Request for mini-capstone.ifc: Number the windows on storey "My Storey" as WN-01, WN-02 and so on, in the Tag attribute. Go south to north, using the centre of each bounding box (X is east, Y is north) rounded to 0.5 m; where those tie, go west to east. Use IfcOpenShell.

First a look at what the model holds.

```python
import ifcopenshell
import ifcopenshell.util.element
import ifcopenshell.util.placement

model = ifcopenshell.open("mini-capstone.ifc")
print(model.schema)
storey = next(s for s in model.by_type("IfcBuildingStorey") if s.Name == "My Storey")
windows = [e for e in ifcopenshell.util.element.get_decomposition(storey) if e.is_a("IfcWindow")]
for e in sorted(windows, key=lambda e: e.id()):
    origin = ifcopenshell.util.placement.get_local_placement(e.ObjectPlacement)[:3, 3]
    print(e.id(), e.Tag, e.Name, origin.round(2) + 0.0, sep=" | ")
```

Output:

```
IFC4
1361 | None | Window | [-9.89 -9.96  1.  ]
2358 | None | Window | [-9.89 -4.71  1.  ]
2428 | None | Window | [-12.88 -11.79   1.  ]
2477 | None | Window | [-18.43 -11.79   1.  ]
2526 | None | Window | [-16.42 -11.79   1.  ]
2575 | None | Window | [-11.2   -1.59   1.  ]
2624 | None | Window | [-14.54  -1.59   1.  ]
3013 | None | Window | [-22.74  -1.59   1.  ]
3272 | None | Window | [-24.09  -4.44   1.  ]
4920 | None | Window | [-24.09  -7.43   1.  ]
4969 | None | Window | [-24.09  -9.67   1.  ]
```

```python
import ifcopenshell
import ifcopenshell.geom
import ifcopenshell.util.element
import ifcopenshell.util.shape

model = ifcopenshell.open("mini-capstone.ifc")
settings = ifcopenshell.geom.settings()
settings.set("use-world-coords", True)


def centre(element):
    shape = ifcopenshell.geom.create_shape(settings, element)
    return ifcopenshell.util.shape.get_bbox_centroid(shape.geometry)


storey = next(s for s in model.by_type("IfcBuildingStorey") if s.Name == "My Storey")
windows = [e for e in ifcopenshell.util.element.get_decomposition(storey) if e.is_a("IfcWindow")]

# Insertion points can sit at a corner or the storey origin, so sort by the geometry (in metres).
centres = {e: centre(e) for e in windows}
windows.sort(key=lambda e: (round(centres[e][1] / 0.5), centres[e][0]))

for i, e in enumerate(windows, start=1):
    number = f"WN-{i:02d}"
    e.Tag = number
    print(e.id(), number)

model.write("mini-capstone_updated.ifc")
```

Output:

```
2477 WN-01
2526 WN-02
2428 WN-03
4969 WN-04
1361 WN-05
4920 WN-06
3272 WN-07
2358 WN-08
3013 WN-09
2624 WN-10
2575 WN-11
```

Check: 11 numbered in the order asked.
